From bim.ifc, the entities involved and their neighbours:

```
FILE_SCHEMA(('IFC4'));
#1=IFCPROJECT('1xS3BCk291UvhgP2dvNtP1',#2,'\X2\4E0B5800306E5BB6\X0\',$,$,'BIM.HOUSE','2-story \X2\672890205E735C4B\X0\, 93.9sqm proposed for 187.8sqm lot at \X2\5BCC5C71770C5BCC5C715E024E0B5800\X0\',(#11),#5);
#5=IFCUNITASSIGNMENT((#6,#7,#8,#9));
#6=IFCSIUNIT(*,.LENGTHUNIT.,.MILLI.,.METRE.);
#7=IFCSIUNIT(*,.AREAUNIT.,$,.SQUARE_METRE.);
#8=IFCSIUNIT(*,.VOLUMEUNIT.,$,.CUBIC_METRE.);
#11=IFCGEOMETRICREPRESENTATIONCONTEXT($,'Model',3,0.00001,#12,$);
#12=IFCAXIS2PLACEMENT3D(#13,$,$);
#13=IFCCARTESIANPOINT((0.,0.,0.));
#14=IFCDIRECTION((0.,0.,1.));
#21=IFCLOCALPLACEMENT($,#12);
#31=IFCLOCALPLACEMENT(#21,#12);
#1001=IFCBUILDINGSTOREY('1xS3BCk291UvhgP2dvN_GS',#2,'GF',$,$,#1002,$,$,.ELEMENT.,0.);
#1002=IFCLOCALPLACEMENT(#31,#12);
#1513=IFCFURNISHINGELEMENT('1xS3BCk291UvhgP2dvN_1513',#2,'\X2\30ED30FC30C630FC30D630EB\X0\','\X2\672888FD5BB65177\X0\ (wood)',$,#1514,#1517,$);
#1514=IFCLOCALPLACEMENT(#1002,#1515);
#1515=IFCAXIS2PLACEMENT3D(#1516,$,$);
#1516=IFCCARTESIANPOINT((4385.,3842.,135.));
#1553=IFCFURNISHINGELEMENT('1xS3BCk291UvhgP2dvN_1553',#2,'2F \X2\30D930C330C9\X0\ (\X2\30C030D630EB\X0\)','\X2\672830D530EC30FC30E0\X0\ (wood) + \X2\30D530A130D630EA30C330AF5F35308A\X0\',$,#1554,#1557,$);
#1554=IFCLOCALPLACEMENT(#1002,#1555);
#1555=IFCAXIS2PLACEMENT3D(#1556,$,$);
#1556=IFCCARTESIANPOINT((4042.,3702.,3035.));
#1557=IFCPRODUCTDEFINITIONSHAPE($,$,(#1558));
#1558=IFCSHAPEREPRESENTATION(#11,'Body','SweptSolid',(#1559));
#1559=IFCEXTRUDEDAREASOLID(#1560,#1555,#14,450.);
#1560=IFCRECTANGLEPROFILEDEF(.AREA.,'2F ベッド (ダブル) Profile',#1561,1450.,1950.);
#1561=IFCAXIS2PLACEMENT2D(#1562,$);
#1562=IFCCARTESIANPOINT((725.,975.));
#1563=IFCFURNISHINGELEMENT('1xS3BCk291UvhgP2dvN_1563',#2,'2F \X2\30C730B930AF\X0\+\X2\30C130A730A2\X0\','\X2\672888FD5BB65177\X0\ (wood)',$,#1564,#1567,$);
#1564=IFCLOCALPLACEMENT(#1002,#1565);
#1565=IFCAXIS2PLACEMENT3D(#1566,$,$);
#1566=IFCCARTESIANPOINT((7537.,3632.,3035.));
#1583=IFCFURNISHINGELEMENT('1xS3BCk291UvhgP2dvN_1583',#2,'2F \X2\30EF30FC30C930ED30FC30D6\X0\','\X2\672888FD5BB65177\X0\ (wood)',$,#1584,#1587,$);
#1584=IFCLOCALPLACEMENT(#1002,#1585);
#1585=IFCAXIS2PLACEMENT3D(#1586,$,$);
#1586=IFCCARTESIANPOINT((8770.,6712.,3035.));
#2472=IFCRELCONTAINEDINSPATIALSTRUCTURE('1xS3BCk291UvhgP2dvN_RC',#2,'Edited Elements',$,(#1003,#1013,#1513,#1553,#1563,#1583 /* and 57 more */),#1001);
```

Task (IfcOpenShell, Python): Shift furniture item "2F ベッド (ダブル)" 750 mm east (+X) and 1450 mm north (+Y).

```python
import ifcopenshell
import ifcopenshell.api.geometry
import ifcopenshell.util.placement
import ifcopenshell.util.unit

model = ifcopenshell.open("bim.ifc")
unit_scale = ifcopenshell.util.unit.calculate_unit_scale(model)

item = model.by_guid("1xS3BCk291UvhgP2dvN_1553")
matrix = ifcopenshell.util.placement.get_local_placement(item.ObjectPlacement)
matrix[0, 3] += 0.75 / unit_scale
matrix[1, 3] += 1.45 / unit_scale
ifcopenshell.api.geometry.edit_object_placement(model, product=item, matrix=matrix, is_si=False)

print(ifcopenshell.util.placement.get_local_placement(item.ObjectPlacement).round(3) + 0.0)

model.write("bim_updated.ifc")
```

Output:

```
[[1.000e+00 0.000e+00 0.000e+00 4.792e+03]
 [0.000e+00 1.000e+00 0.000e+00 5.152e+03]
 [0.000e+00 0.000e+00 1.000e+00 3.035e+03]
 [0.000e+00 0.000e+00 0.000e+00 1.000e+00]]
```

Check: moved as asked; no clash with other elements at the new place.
